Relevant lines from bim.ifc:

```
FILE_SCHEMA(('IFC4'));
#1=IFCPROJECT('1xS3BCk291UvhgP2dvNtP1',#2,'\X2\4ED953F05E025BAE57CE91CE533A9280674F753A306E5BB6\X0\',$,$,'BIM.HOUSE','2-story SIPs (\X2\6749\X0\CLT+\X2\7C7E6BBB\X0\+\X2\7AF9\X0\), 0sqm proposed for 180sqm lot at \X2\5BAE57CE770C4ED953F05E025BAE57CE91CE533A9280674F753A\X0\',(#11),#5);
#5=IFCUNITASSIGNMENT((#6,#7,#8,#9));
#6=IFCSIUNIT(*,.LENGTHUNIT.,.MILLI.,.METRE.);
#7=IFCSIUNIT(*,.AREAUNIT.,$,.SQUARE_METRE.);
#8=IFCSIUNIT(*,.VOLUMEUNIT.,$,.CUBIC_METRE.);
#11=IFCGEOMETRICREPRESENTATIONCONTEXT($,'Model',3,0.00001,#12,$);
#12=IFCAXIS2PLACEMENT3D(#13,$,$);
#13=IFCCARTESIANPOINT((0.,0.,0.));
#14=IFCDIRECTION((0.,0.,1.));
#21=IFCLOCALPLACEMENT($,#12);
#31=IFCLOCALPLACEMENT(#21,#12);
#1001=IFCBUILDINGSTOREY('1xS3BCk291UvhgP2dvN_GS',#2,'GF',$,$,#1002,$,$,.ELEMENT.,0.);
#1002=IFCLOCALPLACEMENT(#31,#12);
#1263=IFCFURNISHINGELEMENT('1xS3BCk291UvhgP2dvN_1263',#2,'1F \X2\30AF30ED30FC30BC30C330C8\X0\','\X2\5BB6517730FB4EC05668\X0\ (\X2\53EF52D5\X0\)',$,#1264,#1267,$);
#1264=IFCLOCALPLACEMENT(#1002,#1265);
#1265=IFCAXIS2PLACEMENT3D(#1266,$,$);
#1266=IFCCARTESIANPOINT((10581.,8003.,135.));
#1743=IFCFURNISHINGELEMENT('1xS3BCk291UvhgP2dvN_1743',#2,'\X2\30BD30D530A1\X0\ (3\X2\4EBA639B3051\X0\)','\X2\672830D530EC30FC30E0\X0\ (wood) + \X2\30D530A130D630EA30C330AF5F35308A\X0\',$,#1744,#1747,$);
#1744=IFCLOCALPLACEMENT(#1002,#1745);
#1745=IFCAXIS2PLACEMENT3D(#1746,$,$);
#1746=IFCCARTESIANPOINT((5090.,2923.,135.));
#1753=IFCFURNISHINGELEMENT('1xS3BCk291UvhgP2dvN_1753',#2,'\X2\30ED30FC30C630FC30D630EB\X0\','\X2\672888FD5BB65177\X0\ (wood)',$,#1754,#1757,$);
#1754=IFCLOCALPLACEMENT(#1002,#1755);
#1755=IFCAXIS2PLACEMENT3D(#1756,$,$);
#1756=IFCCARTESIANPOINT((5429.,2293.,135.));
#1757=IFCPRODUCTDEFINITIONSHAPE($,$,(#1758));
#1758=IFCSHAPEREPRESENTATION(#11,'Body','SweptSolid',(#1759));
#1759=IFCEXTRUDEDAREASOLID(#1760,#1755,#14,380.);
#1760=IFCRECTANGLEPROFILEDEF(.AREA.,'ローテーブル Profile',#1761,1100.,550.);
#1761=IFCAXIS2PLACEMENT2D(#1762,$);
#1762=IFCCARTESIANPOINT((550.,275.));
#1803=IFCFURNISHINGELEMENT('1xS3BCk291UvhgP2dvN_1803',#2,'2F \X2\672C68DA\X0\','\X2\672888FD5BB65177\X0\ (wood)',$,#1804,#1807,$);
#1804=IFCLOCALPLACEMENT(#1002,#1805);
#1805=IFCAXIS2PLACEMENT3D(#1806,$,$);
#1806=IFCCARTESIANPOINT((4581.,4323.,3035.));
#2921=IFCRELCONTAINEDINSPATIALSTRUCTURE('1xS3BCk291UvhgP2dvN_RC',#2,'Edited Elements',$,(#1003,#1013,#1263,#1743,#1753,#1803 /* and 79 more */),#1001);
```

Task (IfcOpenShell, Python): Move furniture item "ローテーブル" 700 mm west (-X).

```python
import ifcopenshell
import ifcopenshell.api.geometry
import ifcopenshell.util.placement

model = ifcopenshell.open("bim.ifc")

item = model.by_guid("1xS3BCk291UvhgP2dvN_1753")
matrix = ifcopenshell.util.placement.get_local_placement(item.ObjectPlacement)
matrix[0, 3] -= 700.0
ifcopenshell.api.geometry.edit_object_placement(model, product=item, matrix=matrix, is_si=False)

print(ifcopenshell.util.placement.get_local_placement(item.ObjectPlacement).round(3) + 0.0)

model.write("bim_v2.ifc")
```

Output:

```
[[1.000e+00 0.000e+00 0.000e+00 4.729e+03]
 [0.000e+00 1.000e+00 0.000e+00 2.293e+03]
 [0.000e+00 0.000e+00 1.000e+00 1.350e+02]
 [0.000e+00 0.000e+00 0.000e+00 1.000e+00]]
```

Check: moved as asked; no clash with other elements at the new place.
